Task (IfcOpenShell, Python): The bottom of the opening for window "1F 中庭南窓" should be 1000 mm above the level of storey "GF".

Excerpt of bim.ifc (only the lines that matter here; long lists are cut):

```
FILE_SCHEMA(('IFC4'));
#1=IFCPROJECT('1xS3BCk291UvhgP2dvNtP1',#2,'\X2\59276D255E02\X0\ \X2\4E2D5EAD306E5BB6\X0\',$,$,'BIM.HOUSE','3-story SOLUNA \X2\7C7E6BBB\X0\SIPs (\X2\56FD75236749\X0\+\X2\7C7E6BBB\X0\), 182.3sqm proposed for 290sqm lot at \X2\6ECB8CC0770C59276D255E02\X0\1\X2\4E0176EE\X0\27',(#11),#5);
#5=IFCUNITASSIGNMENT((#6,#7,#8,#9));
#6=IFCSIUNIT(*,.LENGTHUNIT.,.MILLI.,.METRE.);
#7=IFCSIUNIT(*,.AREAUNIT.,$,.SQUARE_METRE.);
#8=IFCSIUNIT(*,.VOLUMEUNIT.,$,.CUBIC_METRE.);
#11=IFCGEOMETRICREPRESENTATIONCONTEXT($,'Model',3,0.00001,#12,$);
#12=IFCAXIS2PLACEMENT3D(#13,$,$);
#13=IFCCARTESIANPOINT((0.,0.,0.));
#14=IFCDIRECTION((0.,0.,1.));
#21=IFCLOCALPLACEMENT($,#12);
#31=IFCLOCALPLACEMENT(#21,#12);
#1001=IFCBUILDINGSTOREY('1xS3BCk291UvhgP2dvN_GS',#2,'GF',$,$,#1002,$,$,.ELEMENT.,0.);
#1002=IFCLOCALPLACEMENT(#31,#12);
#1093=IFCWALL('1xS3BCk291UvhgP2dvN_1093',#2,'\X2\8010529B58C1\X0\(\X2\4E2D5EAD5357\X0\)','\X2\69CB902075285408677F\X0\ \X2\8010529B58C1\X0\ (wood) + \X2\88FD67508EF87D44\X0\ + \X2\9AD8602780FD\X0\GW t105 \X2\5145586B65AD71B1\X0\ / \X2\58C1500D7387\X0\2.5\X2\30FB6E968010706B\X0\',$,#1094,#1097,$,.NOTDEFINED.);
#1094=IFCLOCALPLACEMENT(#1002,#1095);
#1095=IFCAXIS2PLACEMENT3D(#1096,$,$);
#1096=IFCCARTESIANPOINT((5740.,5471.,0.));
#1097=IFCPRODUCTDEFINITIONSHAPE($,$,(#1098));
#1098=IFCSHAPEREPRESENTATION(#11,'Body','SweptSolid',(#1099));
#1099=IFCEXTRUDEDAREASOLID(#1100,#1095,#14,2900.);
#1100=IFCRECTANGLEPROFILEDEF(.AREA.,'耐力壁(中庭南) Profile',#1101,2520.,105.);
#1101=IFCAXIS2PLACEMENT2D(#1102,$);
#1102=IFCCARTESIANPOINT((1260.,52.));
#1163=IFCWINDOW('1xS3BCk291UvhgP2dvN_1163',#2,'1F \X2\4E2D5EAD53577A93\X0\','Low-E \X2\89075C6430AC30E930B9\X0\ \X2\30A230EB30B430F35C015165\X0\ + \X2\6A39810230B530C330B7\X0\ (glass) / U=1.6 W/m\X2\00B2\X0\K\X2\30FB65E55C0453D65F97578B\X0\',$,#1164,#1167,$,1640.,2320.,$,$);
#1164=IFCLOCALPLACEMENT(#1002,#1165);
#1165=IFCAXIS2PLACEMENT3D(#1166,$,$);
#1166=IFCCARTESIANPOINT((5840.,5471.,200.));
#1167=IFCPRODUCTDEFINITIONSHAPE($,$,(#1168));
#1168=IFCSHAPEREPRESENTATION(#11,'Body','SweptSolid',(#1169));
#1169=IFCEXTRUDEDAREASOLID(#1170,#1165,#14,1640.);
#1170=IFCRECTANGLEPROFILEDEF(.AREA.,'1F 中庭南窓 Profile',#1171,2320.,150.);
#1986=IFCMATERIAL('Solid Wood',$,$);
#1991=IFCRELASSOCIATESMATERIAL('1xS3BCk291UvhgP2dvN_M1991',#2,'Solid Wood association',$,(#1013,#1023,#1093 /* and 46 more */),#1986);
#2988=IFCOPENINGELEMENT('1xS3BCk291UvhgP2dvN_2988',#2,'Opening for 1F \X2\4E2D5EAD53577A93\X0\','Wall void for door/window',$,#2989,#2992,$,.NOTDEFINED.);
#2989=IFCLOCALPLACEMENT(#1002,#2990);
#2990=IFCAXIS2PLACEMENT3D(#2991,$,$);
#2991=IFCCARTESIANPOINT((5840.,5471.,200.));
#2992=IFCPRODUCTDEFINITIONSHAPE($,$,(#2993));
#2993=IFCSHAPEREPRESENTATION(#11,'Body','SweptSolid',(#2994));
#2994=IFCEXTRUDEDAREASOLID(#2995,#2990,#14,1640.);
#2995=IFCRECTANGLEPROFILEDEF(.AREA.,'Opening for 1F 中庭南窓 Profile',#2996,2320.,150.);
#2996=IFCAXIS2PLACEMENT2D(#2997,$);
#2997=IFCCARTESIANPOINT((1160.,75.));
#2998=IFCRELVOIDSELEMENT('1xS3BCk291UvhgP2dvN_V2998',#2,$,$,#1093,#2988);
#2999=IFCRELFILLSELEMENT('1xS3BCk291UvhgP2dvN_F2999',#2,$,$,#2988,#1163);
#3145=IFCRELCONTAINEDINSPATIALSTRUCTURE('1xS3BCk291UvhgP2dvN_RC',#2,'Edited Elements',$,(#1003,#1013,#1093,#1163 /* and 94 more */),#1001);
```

```python
import numpy as np
import ifcopenshell
import ifcopenshell.api.geometry
import ifcopenshell.geom
import ifcopenshell.util.element
import ifcopenshell.util.placement
import ifcopenshell.util.shape
import ifcopenshell.util.unit

model = ifcopenshell.open("bim.ifc")
unit_scale = ifcopenshell.util.unit.calculate_unit_scale(model)

window = model.by_id(1163)
opening = window.FillsVoids[0].RelatingOpeningElement
storey = ifcopenshell.util.element.get_container(window, ifc_class="IfcBuildingStorey")
level = ifcopenshell.util.placement.get_local_placement(storey.ObjectPlacement)[2, 3]

# The opening's origin need not be at the sill, so measure its lowest point.
shape = ifcopenshell.geom.create_shape(ifcopenshell.geom.settings(), opening)
bottom = ifcopenshell.util.shape.get_shape_bottom_elevation(shape, shape.geometry) / unit_scale
dz = level + 1000.0 - bottom

shift = np.array([0.0, 0.0, dz])
# The window is not placed relative to its opening, so move both.
for product in (opening, window):
    matrix = ifcopenshell.util.placement.get_local_placement(product.ObjectPlacement)
    matrix[:3, 3] += shift
    ifcopenshell.api.geometry.edit_object_placement(model, product=product, matrix=matrix, is_si=False)

print(f"moved by {dz * unit_scale:+.3f} m")

model.write("bim_rev.ifc")
```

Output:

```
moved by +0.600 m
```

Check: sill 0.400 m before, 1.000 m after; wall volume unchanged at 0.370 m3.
